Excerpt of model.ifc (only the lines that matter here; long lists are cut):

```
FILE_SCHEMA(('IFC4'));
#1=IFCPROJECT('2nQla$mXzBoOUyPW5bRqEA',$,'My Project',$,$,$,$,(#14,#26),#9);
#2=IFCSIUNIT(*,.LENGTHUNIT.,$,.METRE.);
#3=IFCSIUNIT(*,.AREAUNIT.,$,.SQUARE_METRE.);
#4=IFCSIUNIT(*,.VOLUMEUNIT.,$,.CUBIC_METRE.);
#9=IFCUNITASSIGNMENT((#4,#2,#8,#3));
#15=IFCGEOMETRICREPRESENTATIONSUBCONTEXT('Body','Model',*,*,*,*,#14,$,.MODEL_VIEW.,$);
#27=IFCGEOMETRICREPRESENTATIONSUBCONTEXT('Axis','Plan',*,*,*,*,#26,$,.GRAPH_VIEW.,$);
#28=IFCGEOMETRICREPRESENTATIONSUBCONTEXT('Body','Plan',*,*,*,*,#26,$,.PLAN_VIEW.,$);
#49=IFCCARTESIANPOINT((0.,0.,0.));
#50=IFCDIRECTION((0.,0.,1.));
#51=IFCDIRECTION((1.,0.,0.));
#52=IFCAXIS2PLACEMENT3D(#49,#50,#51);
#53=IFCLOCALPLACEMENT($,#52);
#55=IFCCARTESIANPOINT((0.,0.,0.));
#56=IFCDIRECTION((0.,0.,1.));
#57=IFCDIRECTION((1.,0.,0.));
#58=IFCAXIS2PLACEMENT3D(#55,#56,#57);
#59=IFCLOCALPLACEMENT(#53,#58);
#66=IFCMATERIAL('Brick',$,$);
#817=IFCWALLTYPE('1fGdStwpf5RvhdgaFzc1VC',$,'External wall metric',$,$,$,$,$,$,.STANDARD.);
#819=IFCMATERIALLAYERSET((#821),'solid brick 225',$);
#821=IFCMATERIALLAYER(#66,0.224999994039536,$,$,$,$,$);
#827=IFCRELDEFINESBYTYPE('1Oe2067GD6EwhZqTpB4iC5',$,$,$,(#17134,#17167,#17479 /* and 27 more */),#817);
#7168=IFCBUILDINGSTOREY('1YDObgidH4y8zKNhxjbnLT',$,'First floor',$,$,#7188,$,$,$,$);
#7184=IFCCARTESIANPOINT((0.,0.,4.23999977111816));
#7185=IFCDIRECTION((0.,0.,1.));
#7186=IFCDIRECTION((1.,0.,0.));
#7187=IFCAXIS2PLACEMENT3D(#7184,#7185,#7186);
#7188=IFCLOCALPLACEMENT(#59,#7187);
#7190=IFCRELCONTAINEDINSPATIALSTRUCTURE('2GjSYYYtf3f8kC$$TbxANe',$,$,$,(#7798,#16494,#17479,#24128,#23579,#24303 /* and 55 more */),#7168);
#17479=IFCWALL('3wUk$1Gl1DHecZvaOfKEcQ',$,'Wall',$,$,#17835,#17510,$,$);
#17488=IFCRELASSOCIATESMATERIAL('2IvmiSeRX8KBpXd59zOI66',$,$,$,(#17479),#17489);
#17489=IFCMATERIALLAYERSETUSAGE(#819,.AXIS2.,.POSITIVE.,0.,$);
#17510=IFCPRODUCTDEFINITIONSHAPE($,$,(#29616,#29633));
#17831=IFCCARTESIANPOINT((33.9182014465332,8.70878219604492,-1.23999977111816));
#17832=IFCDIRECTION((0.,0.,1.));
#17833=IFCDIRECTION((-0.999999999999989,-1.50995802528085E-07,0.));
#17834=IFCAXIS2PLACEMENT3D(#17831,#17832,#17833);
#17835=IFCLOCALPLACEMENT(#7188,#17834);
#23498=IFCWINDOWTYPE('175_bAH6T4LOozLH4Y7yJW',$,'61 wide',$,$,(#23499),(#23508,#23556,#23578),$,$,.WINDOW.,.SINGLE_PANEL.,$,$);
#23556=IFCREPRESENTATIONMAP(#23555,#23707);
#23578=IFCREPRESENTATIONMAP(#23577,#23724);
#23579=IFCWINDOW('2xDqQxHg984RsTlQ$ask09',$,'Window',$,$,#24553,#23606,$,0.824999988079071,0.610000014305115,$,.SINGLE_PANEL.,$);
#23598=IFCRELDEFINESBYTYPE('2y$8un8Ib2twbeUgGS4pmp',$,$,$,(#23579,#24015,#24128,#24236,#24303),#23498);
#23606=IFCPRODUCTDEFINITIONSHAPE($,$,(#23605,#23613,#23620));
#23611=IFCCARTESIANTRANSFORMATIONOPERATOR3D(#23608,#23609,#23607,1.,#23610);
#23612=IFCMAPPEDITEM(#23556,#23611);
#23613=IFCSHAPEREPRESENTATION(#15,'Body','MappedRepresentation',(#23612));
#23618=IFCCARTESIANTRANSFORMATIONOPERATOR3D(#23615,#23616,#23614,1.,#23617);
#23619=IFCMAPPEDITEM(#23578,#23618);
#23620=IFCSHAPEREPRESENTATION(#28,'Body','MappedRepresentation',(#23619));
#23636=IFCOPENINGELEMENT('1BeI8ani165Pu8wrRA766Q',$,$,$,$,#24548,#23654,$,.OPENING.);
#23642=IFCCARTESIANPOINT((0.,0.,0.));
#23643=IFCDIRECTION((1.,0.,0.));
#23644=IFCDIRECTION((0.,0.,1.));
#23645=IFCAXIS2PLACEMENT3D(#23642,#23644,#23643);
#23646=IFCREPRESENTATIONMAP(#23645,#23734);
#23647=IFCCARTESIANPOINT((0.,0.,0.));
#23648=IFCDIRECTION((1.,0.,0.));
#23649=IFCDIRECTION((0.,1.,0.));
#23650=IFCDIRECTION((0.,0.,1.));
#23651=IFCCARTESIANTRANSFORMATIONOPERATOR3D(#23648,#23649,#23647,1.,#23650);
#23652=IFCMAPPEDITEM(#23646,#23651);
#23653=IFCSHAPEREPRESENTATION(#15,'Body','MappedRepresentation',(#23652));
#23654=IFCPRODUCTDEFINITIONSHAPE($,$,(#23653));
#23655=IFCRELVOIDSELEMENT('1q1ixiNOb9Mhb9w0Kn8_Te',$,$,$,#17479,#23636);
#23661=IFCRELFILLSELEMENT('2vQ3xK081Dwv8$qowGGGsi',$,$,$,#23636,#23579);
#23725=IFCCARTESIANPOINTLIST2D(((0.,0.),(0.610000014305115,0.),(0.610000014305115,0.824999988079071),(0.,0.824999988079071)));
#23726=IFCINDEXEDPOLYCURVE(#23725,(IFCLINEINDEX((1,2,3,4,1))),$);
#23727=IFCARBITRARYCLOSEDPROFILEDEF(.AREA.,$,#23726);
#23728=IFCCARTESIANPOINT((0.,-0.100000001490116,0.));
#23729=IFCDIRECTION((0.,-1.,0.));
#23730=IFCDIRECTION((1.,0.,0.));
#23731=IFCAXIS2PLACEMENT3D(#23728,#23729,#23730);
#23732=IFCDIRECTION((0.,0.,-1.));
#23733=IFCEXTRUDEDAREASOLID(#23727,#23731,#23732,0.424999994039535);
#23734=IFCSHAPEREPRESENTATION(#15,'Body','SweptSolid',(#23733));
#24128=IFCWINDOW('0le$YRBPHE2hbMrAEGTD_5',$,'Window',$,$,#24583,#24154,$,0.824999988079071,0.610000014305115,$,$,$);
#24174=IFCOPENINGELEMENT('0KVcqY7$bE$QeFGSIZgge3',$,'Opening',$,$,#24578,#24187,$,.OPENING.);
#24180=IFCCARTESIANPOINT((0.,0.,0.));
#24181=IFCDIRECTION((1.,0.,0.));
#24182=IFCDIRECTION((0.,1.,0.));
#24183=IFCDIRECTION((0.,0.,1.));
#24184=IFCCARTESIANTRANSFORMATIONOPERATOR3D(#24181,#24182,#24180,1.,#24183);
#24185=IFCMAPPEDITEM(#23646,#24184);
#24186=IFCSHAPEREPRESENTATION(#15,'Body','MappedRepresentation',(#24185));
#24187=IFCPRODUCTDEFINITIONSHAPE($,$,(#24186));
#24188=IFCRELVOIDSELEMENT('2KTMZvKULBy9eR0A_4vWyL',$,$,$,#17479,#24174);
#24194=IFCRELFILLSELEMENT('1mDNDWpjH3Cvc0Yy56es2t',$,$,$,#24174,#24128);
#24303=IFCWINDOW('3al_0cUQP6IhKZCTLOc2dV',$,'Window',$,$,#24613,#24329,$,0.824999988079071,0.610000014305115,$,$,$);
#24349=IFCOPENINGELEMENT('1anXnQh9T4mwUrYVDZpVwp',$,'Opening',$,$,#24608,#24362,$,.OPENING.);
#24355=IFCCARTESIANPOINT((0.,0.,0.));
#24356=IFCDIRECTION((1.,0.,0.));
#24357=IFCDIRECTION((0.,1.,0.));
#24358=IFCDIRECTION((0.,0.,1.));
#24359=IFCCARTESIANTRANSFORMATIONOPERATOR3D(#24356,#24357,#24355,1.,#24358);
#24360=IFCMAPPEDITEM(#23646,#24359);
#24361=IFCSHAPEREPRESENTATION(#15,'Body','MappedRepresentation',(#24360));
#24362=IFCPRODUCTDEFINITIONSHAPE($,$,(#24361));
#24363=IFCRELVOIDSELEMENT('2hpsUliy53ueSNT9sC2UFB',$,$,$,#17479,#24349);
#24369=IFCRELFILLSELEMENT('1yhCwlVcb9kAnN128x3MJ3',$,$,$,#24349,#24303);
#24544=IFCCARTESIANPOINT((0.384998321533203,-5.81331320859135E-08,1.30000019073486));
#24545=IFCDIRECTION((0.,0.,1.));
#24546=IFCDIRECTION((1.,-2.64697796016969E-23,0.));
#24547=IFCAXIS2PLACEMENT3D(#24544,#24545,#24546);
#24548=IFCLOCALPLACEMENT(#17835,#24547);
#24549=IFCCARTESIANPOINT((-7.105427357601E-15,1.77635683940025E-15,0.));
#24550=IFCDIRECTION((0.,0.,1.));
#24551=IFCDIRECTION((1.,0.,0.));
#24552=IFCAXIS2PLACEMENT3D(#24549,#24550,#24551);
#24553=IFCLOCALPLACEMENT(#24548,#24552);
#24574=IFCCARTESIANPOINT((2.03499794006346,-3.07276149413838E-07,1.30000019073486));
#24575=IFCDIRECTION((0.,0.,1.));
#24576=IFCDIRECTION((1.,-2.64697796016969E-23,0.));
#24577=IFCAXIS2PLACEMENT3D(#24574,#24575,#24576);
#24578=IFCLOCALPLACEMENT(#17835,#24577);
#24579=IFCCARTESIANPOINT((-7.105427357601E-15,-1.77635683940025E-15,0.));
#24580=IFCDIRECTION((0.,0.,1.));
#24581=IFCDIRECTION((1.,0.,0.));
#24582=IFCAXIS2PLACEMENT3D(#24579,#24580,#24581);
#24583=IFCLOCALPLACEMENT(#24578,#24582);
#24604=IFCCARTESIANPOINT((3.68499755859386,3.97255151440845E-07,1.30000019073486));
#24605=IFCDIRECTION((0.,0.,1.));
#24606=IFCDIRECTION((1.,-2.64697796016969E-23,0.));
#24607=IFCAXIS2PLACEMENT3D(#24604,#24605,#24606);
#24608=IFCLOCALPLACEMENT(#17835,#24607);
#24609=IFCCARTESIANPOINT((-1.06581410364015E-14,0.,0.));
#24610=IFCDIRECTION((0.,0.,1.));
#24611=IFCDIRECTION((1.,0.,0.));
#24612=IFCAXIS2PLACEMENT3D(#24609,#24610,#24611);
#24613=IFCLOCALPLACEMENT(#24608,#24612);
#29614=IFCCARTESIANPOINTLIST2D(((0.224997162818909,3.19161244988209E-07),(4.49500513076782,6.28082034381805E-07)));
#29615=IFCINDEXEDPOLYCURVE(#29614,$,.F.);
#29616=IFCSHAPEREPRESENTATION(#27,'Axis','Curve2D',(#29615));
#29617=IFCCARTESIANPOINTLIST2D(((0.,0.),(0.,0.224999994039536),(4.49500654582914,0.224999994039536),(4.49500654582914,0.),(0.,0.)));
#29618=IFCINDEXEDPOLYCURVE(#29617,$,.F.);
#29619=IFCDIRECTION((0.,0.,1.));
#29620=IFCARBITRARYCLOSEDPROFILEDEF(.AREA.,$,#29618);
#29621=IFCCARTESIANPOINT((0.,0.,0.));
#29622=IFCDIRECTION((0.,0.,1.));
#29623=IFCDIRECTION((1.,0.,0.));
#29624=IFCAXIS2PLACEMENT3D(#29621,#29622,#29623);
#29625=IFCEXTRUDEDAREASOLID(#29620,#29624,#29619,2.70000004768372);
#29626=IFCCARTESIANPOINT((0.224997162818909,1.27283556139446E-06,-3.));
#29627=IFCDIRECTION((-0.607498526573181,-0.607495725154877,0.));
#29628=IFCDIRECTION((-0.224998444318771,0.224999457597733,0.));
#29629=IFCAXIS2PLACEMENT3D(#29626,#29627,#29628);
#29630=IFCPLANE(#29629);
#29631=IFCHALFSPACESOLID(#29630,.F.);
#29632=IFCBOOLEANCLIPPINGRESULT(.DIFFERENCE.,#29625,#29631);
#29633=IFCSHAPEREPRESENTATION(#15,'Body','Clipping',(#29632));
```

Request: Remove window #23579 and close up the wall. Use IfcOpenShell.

```python
import ifcopenshell
import ifcopenshell.api.feature
import ifcopenshell.api.root
import ifcopenshell.geom
import ifcopenshell.util.shape

model = ifcopenshell.open("model.ifc")
settings = ifcopenshell.geom.settings()


def volume(element):
    """Net volume in cubic metres, openings subtracted."""
    shape = ifcopenshell.geom.create_shape(settings, element)
    return ifcopenshell.util.shape.get_volume(shape.geometry)


window = model.by_guid("2xDqQxHg984RsTlQ$ask09")
opening = window.FillsVoids[0].RelatingOpeningElement
wall = opening.VoidsElements[0].RelatingBuildingElement
before = volume(wall)

ifcopenshell.api.root.remove_product(model, product=window)
ifcopenshell.api.feature.remove_feature(model, feature=opening)

after = volume(wall)

print(f"wall volume {before:.3f} -> {after:.3f} m3")

model.write("model_v2.ifc")
```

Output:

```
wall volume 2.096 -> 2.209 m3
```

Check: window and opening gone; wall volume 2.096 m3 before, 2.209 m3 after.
